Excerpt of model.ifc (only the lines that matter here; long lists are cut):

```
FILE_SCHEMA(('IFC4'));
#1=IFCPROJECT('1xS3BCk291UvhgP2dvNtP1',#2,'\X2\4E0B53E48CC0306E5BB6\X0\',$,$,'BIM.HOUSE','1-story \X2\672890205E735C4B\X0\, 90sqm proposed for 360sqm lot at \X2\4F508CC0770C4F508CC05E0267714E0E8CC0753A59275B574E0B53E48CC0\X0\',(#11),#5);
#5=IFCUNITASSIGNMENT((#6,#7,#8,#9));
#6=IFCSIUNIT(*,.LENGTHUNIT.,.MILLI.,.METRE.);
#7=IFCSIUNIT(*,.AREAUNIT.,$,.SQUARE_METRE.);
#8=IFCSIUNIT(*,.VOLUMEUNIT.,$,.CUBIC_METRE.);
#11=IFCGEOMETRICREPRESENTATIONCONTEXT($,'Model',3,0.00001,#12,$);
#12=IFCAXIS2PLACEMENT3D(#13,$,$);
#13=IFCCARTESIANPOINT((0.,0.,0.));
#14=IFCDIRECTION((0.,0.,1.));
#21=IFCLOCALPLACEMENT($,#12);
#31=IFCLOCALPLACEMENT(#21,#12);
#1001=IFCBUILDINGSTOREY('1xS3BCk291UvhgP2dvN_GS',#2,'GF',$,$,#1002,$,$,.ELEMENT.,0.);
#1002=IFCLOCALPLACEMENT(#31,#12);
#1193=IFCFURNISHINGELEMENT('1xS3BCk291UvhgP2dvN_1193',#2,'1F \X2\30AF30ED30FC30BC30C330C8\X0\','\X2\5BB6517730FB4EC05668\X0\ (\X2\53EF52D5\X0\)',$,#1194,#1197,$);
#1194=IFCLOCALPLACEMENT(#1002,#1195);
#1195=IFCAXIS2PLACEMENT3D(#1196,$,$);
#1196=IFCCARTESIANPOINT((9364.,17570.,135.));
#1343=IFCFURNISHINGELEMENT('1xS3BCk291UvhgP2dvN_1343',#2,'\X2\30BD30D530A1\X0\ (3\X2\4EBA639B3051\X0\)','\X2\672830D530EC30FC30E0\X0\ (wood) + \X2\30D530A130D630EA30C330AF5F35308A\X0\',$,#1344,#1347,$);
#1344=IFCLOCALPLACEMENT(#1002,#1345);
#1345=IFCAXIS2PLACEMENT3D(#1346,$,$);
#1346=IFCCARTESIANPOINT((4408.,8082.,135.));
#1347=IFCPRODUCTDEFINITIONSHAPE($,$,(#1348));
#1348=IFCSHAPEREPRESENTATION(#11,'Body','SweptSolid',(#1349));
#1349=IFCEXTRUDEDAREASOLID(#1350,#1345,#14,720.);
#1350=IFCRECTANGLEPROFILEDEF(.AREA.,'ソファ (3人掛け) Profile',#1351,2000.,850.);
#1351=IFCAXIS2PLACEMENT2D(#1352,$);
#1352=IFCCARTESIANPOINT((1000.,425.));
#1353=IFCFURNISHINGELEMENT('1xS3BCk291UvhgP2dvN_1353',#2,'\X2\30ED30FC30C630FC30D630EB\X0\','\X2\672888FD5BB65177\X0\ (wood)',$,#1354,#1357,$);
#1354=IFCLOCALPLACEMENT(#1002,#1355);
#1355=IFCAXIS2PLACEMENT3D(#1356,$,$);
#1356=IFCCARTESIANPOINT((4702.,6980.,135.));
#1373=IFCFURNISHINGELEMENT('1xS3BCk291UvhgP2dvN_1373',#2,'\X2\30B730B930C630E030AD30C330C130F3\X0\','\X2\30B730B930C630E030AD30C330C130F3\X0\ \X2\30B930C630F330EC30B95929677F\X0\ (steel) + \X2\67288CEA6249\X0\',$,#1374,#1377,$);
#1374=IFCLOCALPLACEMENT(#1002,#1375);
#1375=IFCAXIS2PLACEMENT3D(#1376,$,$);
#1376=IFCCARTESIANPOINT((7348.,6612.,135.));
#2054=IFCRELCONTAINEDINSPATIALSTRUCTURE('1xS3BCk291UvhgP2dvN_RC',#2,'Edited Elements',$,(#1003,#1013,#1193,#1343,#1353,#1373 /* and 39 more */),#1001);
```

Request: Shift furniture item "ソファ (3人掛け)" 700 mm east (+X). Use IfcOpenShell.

```python
import ifcopenshell
import ifcopenshell.api.geometry
import ifcopenshell.util.placement
import ifcopenshell.util.unit

model = ifcopenshell.open("model.ifc")
unit_scale = ifcopenshell.util.unit.calculate_unit_scale(model)

item = model.by_guid("1xS3BCk291UvhgP2dvN_1343")
matrix = ifcopenshell.util.placement.get_local_placement(item.ObjectPlacement)
matrix[0, 3] += 0.7 / unit_scale
ifcopenshell.api.geometry.edit_object_placement(model, product=item, matrix=matrix, is_si=False)

print(ifcopenshell.util.placement.get_local_placement(item.ObjectPlacement).round(3) + 0.0)

model.write("model_edited.ifc")
```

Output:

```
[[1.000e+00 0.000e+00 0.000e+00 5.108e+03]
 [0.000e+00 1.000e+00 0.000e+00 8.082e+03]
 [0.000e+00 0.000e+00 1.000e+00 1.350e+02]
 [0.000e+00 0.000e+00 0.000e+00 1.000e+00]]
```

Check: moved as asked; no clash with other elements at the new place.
